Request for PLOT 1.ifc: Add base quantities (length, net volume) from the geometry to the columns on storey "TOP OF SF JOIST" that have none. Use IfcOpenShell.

First a look at what the model holds.

```python
import ifcopenshell
import ifcopenshell.util.element
import ifcopenshell.util.unit

model = ifcopenshell.open("PLOT 1.ifc")
print(model.schema)
for unit_type in ("LENGTHUNIT", "AREAUNIT", "VOLUMEUNIT"):
    print(unit_type, ifcopenshell.util.unit.calculate_unit_scale(model, unit_type))
storey = next(s for s in model.by_type("IfcBuildingStorey") if s.Name == "TOP OF SF JOIST")
columns = [e for e in ifcopenshell.util.element.get_decomposition(storey) if e.is_a("IfcColumn")]
for e in sorted(columns, key=lambda e: e.id()):
    print(e.id(), e.is_a(), e.Name, list(ifcopenshell.util.element.get_psets(e, qtos_only=True)), sep=" | ")
```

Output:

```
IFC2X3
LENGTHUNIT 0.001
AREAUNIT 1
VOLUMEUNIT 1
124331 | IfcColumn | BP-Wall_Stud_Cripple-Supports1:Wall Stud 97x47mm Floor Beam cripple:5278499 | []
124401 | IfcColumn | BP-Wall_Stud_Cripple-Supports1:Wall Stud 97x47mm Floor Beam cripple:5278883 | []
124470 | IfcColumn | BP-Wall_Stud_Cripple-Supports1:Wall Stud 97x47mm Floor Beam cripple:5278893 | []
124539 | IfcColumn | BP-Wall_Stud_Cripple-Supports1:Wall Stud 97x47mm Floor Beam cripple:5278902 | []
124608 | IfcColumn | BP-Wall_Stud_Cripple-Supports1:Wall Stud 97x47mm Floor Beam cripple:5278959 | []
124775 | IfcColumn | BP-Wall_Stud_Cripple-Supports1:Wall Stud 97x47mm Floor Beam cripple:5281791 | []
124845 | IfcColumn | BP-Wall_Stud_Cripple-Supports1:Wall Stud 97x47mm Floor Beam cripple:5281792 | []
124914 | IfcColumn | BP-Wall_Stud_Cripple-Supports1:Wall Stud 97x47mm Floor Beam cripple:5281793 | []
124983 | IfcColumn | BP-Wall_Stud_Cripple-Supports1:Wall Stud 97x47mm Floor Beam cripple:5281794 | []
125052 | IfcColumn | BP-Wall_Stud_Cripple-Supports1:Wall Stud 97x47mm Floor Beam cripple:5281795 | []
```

```python
import ifcopenshell
import ifcopenshell.api.pset
import ifcopenshell.geom
import ifcopenshell.util.element
import ifcopenshell.util.shape
import ifcopenshell.util.unit

model = ifcopenshell.open("PLOT 1.ifc")
unit_scale = ifcopenshell.util.unit.calculate_unit_scale(model)
volume_scale = ifcopenshell.util.unit.calculate_unit_scale(model, "VOLUMEUNIT")
settings = ifcopenshell.geom.settings()

storey = next(s for s in model.by_type("IfcBuildingStorey") if s.Name == "TOP OF SF JOIST")
columns = [e for e in ifcopenshell.util.element.get_decomposition(storey) if e.is_a("IfcColumn")]

for e in sorted(columns, key=lambda e: e.id()):
    if ifcopenshell.util.element.get_psets(e, qtos_only=True, should_inherit=False):
        continue
    # Geometry comes back in metres, in the element's own axes.
    shape = ifcopenshell.geom.create_shape(settings, e)
    values = {
        "Length": ifcopenshell.util.shape.get_z(shape.geometry) / unit_scale,
        "NetVolume": ifcopenshell.util.shape.get_volume(shape.geometry) / volume_scale,
    }
    qto = ifcopenshell.api.pset.add_qto(model, product=e, name="BaseQuantities")
    ifcopenshell.api.pset.edit_qto(model, qto=qto, properties=values)
    print(e.id(), {k: round(v, 3) for k, v in values.items()})

model.write("PLOT 1_edited.ifc")
```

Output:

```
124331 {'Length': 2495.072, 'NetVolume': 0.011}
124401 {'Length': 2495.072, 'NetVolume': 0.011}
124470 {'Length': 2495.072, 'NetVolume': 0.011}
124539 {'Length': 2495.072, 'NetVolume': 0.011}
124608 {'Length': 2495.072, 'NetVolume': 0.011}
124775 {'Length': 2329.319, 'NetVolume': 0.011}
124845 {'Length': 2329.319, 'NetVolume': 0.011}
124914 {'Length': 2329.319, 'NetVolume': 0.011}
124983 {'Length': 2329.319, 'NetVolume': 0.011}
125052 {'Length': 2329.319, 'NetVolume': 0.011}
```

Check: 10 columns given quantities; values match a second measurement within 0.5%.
